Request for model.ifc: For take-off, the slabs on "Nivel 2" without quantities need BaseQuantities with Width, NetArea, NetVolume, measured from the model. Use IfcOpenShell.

First a look at what the model holds.

```python
import ifcopenshell
import ifcopenshell.util.element
import ifcopenshell.util.unit

model = ifcopenshell.open("model.ifc")
print(model.schema)
for unit_type in ("LENGTHUNIT", "AREAUNIT", "VOLUMEUNIT"):
    print(unit_type, ifcopenshell.util.unit.calculate_unit_scale(model, unit_type))
storey = next(s for s in model.by_type("IfcBuildingStorey") if s.Name == "Nivel 2")
slabs = [e for e in ifcopenshell.util.element.get_decomposition(storey) if e.is_a("IfcSlab")]
for e in sorted(slabs, key=lambda e: e.id()):
    print(e.id(), e.is_a(), e.Name, list(ifcopenshell.util.element.get_psets(e, qtos_only=True)), sep=" | ")
```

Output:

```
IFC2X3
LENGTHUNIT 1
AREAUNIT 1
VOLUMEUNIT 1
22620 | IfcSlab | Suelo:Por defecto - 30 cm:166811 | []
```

```python
import ifcopenshell
import ifcopenshell.api.pset
import ifcopenshell.geom
import ifcopenshell.util.element
import ifcopenshell.util.shape
import ifcopenshell.util.unit

model = ifcopenshell.open("model.ifc")
unit_scale = ifcopenshell.util.unit.calculate_unit_scale(model)
area_scale = ifcopenshell.util.unit.calculate_unit_scale(model, "AREAUNIT")
volume_scale = ifcopenshell.util.unit.calculate_unit_scale(model, "VOLUMEUNIT")
settings = ifcopenshell.geom.settings()

storey = next(s for s in model.by_type("IfcBuildingStorey") if s.Name == "Nivel 2")
slabs = [e for e in ifcopenshell.util.element.get_decomposition(storey) if e.is_a("IfcSlab")]

for e in sorted(slabs, key=lambda e: e.id()):
    if ifcopenshell.util.element.get_psets(e, qtos_only=True, should_inherit=False):
        continue
    # Geometry comes back in metres, in the element's own axes.
    shape = ifcopenshell.geom.create_shape(settings, e)
    values = {
        "Width": ifcopenshell.util.shape.get_z(shape.geometry) / unit_scale,
        "NetArea": ifcopenshell.util.shape.get_footprint_area(shape.geometry) / area_scale,
        "NetVolume": ifcopenshell.util.shape.get_volume(shape.geometry) / volume_scale,
    }
    qto = ifcopenshell.api.pset.add_qto(model, product=e, name="BaseQuantities")
    ifcopenshell.api.pset.edit_qto(model, qto=qto, properties=values)
    print(e.id(), {k: round(v, 3) for k, v in values.items()})

model.write("model_updated.ifc")
```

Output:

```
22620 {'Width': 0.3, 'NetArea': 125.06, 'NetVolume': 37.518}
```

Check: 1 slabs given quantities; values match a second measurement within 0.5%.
